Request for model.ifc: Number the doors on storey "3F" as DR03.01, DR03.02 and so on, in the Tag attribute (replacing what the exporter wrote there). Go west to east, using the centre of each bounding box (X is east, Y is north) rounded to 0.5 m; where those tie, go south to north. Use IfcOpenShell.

First a look at what the model holds.

```python
import ifcopenshell
import ifcopenshell.util.element
import ifcopenshell.util.placement

model = ifcopenshell.open("model.ifc")
print(model.schema)
storey = next(s for s in model.by_type("IfcBuildingStorey") if s.Name == "3F")
doors = [e for e in ifcopenshell.util.element.get_decomposition(storey) if e.is_a("IfcDoor")]
for e in sorted(doors, key=lambda e: e.id()):
    origin = ifcopenshell.util.placement.get_local_placement(e.ObjectPlacement)[:3, 3]
    print(e.id(), e.Tag, e.Name, origin.round(2) + 0.0, sep=" | ")
```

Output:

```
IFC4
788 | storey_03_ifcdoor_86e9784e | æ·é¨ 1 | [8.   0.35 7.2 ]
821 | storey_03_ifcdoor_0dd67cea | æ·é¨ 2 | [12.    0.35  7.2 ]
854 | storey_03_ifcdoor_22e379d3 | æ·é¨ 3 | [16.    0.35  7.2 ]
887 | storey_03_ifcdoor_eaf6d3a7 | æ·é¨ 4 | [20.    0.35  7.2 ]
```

```python
import ifcopenshell
import ifcopenshell.geom
import ifcopenshell.util.element
import ifcopenshell.util.shape

model = ifcopenshell.open("model.ifc")
settings = ifcopenshell.geom.settings()
settings.set("use-world-coords", True)


def centre(element):
    shape = ifcopenshell.geom.create_shape(settings, element)
    return ifcopenshell.util.shape.get_bbox_centroid(shape.geometry)


storey = next(s for s in model.by_type("IfcBuildingStorey") if s.Name == "3F")
doors = [e for e in ifcopenshell.util.element.get_decomposition(storey) if e.is_a("IfcDoor")]

# Insertion points can sit at a corner or the storey origin, so sort by the geometry (in metres).
centres = {e: centre(e) for e in doors}
doors.sort(key=lambda e: (round(centres[e][0] / 0.5), centres[e][1]))

for i, e in enumerate(doors, start=1):
    number = f"DR03.{i:02d}"
    e.Tag = number
    print(e.id(), number)

model.write("model_v2.ifc")
```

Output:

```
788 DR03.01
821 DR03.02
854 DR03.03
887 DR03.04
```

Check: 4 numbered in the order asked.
